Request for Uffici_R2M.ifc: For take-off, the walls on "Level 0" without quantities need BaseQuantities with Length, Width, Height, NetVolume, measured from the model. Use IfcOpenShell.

First a look at what the model holds.

```python
import ifcopenshell
import ifcopenshell.util.element
import ifcopenshell.util.unit

model = ifcopenshell.open("Uffici_R2M.ifc")
print(model.schema)
for unit_type in ("LENGTHUNIT", "AREAUNIT", "VOLUMEUNIT"):
    print(unit_type, ifcopenshell.util.unit.calculate_unit_scale(model, unit_type))
storey = next(s for s in model.by_type("IfcBuildingStorey") if s.Name == "Level 0")
walls = [e for e in ifcopenshell.util.element.get_decomposition(storey) if e.is_a("IfcWall")]
for e in sorted(walls, key=lambda e: e.id()):
    print(e.id(), e.is_a(), e.Name, list(ifcopenshell.util.element.get_psets(e, qtos_only=True)), sep=" | ")
```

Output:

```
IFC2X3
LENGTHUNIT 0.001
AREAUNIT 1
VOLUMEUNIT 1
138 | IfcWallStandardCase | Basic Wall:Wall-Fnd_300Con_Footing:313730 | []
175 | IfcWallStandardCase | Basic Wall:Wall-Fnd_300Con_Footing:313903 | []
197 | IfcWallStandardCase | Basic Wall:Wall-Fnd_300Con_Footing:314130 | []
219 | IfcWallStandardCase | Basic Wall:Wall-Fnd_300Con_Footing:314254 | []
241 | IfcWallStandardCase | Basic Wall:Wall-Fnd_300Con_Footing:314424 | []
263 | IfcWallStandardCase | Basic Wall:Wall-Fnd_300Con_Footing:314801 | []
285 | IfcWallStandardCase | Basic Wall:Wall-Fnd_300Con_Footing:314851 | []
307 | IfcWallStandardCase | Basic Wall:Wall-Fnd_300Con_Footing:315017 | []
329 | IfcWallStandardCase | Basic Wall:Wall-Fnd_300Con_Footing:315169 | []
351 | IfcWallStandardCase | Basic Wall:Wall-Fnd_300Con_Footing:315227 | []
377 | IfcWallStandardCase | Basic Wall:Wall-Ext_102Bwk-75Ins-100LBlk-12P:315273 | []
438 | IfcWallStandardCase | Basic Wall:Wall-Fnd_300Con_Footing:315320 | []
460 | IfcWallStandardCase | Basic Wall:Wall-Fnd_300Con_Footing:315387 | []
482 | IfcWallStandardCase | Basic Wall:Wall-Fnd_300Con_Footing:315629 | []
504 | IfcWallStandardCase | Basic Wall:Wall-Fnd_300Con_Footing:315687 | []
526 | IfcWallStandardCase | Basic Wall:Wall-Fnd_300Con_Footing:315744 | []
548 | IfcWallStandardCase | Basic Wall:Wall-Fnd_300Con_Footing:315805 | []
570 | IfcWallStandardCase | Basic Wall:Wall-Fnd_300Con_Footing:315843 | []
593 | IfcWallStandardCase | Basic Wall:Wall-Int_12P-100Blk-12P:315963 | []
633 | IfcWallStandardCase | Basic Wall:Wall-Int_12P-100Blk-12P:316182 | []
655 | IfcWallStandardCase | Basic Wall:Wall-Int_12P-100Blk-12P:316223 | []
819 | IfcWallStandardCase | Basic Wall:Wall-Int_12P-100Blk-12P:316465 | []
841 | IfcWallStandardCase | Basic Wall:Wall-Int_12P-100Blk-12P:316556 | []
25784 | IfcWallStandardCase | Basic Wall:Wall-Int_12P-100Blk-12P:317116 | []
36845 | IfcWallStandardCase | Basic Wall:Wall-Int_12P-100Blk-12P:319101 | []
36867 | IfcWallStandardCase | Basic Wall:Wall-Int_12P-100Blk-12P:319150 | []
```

```python
import ifcopenshell
import ifcopenshell.api.pset
import ifcopenshell.geom
import ifcopenshell.util.element
import ifcopenshell.util.shape
import ifcopenshell.util.unit

model = ifcopenshell.open("Uffici_R2M.ifc")
unit_scale = ifcopenshell.util.unit.calculate_unit_scale(model)
volume_scale = ifcopenshell.util.unit.calculate_unit_scale(model, "VOLUMEUNIT")
settings = ifcopenshell.geom.settings()

storey = next(s for s in model.by_type("IfcBuildingStorey") if s.Name == "Level 0")
walls = [e for e in ifcopenshell.util.element.get_decomposition(storey) if e.is_a("IfcWall")]

for e in sorted(walls, key=lambda e: e.id()):
    if ifcopenshell.util.element.get_psets(e, qtos_only=True, should_inherit=False):
        continue
    # Geometry comes back in metres, in the element's own axes.
    shape = ifcopenshell.geom.create_shape(settings, e)
    values = {
        "Length": ifcopenshell.util.shape.get_x(shape.geometry) / unit_scale,
        "Width": ifcopenshell.util.shape.get_y(shape.geometry) / unit_scale,
        "Height": ifcopenshell.util.shape.get_z(shape.geometry) / unit_scale,
        "NetVolume": ifcopenshell.util.shape.get_volume(shape.geometry) / volume_scale,
    }
    qto = ifcopenshell.api.pset.add_qto(model, product=e, name="BaseQuantities")
    ifcopenshell.api.pset.edit_qto(model, qto=qto, properties=values)
    print(e.id(), {k: round(v, 3) for k, v in values.items()})

model.write("Uffici_R2M-out.ifc")
```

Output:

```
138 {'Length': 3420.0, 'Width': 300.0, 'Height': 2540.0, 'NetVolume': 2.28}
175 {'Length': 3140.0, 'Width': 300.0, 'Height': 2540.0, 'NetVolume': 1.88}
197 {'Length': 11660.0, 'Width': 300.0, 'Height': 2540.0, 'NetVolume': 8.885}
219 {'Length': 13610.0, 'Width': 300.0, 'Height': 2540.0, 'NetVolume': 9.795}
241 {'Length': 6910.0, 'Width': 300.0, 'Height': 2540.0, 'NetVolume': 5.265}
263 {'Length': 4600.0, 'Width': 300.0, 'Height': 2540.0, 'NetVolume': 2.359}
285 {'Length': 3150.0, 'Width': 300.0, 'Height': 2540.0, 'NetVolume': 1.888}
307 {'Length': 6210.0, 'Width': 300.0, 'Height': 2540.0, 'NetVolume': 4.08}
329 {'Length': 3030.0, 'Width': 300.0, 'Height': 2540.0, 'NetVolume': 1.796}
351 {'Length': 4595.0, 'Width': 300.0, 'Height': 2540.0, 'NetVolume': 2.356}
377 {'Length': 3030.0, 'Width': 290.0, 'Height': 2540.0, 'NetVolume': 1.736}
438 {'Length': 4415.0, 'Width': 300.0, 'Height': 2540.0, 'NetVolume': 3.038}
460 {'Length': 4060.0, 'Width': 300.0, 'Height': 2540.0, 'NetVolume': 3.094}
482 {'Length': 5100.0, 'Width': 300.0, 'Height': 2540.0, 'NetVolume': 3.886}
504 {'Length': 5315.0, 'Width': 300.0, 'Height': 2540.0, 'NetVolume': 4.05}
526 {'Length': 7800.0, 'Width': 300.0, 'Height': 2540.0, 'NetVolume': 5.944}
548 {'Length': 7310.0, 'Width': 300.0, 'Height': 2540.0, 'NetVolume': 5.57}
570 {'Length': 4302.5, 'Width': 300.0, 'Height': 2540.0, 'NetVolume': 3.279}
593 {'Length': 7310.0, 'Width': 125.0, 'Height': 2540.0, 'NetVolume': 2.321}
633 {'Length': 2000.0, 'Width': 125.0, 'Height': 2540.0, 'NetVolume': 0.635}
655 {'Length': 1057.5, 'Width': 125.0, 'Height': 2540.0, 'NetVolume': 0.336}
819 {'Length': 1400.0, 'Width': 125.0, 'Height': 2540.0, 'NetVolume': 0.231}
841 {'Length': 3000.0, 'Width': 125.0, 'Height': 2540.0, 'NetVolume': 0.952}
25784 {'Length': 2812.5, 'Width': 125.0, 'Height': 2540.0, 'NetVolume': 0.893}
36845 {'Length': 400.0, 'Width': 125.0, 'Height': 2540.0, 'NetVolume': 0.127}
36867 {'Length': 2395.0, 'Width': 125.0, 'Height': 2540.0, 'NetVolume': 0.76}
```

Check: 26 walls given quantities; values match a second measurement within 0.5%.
